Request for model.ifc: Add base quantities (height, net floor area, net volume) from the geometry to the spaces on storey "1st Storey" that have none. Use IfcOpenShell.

First a look at what the model holds.

```python
import ifcopenshell
import ifcopenshell.util.element
import ifcopenshell.util.unit

model = ifcopenshell.open("model.ifc")
print(model.schema)
for unit_type in ("LENGTHUNIT", "AREAUNIT", "VOLUMEUNIT"):
    print(unit_type, ifcopenshell.util.unit.calculate_unit_scale(model, unit_type))
storey = next(s for s in model.by_type("IfcBuildingStorey") if s.Name == "1st Storey")
spaces = [e for e in ifcopenshell.util.element.get_decomposition(storey) if e.is_a("IfcSpace")]
for e in sorted(spaces, key=lambda e: e.id()):
    print(e.id(), e.is_a(), e.Name, list(ifcopenshell.util.element.get_psets(e, qtos_only=True)), sep=" | ")
```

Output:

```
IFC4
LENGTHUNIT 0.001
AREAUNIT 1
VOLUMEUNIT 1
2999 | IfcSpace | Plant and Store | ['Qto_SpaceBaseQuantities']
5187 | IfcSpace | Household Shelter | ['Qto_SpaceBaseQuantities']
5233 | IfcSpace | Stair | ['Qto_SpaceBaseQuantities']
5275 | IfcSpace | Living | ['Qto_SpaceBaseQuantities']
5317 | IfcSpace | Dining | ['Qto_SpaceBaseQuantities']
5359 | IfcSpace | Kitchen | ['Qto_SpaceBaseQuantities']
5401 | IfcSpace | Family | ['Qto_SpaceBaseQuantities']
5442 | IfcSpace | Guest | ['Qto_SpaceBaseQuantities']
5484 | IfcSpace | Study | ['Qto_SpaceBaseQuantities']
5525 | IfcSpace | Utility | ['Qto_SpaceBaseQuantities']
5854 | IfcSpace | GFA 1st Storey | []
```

```python
import ifcopenshell
import ifcopenshell.api.pset
import ifcopenshell.geom
import ifcopenshell.util.element
import ifcopenshell.util.shape
import ifcopenshell.util.unit

model = ifcopenshell.open("model.ifc")
unit_scale = ifcopenshell.util.unit.calculate_unit_scale(model)
area_scale = ifcopenshell.util.unit.calculate_unit_scale(model, "AREAUNIT")
volume_scale = ifcopenshell.util.unit.calculate_unit_scale(model, "VOLUMEUNIT")
settings = ifcopenshell.geom.settings()

storey = next(s for s in model.by_type("IfcBuildingStorey") if s.Name == "1st Storey")
spaces = [e for e in ifcopenshell.util.element.get_decomposition(storey) if e.is_a("IfcSpace")]

for e in sorted(spaces, key=lambda e: e.id()):
    if ifcopenshell.util.element.get_psets(e, qtos_only=True, should_inherit=False):
        continue
    # Geometry comes back in metres, in the element's own axes.
    shape = ifcopenshell.geom.create_shape(settings, e)
    values = {
        "Height": ifcopenshell.util.shape.get_z(shape.geometry) / unit_scale,
        "NetFloorArea": ifcopenshell.util.shape.get_footprint_area(shape.geometry) / area_scale,
        "NetVolume": ifcopenshell.util.shape.get_volume(shape.geometry) / volume_scale,
    }
    qto = ifcopenshell.api.pset.add_qto(model, product=e, name="Qto_SpaceBaseQuantities")
    ifcopenshell.api.pset.edit_qto(model, qto=qto, properties=values)
    print(e.id(), {k: round(v, 3) for k, v in values.items()})

model.write("model_edited.ifc")
```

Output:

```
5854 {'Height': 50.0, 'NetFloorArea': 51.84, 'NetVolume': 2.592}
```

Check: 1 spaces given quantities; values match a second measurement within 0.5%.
